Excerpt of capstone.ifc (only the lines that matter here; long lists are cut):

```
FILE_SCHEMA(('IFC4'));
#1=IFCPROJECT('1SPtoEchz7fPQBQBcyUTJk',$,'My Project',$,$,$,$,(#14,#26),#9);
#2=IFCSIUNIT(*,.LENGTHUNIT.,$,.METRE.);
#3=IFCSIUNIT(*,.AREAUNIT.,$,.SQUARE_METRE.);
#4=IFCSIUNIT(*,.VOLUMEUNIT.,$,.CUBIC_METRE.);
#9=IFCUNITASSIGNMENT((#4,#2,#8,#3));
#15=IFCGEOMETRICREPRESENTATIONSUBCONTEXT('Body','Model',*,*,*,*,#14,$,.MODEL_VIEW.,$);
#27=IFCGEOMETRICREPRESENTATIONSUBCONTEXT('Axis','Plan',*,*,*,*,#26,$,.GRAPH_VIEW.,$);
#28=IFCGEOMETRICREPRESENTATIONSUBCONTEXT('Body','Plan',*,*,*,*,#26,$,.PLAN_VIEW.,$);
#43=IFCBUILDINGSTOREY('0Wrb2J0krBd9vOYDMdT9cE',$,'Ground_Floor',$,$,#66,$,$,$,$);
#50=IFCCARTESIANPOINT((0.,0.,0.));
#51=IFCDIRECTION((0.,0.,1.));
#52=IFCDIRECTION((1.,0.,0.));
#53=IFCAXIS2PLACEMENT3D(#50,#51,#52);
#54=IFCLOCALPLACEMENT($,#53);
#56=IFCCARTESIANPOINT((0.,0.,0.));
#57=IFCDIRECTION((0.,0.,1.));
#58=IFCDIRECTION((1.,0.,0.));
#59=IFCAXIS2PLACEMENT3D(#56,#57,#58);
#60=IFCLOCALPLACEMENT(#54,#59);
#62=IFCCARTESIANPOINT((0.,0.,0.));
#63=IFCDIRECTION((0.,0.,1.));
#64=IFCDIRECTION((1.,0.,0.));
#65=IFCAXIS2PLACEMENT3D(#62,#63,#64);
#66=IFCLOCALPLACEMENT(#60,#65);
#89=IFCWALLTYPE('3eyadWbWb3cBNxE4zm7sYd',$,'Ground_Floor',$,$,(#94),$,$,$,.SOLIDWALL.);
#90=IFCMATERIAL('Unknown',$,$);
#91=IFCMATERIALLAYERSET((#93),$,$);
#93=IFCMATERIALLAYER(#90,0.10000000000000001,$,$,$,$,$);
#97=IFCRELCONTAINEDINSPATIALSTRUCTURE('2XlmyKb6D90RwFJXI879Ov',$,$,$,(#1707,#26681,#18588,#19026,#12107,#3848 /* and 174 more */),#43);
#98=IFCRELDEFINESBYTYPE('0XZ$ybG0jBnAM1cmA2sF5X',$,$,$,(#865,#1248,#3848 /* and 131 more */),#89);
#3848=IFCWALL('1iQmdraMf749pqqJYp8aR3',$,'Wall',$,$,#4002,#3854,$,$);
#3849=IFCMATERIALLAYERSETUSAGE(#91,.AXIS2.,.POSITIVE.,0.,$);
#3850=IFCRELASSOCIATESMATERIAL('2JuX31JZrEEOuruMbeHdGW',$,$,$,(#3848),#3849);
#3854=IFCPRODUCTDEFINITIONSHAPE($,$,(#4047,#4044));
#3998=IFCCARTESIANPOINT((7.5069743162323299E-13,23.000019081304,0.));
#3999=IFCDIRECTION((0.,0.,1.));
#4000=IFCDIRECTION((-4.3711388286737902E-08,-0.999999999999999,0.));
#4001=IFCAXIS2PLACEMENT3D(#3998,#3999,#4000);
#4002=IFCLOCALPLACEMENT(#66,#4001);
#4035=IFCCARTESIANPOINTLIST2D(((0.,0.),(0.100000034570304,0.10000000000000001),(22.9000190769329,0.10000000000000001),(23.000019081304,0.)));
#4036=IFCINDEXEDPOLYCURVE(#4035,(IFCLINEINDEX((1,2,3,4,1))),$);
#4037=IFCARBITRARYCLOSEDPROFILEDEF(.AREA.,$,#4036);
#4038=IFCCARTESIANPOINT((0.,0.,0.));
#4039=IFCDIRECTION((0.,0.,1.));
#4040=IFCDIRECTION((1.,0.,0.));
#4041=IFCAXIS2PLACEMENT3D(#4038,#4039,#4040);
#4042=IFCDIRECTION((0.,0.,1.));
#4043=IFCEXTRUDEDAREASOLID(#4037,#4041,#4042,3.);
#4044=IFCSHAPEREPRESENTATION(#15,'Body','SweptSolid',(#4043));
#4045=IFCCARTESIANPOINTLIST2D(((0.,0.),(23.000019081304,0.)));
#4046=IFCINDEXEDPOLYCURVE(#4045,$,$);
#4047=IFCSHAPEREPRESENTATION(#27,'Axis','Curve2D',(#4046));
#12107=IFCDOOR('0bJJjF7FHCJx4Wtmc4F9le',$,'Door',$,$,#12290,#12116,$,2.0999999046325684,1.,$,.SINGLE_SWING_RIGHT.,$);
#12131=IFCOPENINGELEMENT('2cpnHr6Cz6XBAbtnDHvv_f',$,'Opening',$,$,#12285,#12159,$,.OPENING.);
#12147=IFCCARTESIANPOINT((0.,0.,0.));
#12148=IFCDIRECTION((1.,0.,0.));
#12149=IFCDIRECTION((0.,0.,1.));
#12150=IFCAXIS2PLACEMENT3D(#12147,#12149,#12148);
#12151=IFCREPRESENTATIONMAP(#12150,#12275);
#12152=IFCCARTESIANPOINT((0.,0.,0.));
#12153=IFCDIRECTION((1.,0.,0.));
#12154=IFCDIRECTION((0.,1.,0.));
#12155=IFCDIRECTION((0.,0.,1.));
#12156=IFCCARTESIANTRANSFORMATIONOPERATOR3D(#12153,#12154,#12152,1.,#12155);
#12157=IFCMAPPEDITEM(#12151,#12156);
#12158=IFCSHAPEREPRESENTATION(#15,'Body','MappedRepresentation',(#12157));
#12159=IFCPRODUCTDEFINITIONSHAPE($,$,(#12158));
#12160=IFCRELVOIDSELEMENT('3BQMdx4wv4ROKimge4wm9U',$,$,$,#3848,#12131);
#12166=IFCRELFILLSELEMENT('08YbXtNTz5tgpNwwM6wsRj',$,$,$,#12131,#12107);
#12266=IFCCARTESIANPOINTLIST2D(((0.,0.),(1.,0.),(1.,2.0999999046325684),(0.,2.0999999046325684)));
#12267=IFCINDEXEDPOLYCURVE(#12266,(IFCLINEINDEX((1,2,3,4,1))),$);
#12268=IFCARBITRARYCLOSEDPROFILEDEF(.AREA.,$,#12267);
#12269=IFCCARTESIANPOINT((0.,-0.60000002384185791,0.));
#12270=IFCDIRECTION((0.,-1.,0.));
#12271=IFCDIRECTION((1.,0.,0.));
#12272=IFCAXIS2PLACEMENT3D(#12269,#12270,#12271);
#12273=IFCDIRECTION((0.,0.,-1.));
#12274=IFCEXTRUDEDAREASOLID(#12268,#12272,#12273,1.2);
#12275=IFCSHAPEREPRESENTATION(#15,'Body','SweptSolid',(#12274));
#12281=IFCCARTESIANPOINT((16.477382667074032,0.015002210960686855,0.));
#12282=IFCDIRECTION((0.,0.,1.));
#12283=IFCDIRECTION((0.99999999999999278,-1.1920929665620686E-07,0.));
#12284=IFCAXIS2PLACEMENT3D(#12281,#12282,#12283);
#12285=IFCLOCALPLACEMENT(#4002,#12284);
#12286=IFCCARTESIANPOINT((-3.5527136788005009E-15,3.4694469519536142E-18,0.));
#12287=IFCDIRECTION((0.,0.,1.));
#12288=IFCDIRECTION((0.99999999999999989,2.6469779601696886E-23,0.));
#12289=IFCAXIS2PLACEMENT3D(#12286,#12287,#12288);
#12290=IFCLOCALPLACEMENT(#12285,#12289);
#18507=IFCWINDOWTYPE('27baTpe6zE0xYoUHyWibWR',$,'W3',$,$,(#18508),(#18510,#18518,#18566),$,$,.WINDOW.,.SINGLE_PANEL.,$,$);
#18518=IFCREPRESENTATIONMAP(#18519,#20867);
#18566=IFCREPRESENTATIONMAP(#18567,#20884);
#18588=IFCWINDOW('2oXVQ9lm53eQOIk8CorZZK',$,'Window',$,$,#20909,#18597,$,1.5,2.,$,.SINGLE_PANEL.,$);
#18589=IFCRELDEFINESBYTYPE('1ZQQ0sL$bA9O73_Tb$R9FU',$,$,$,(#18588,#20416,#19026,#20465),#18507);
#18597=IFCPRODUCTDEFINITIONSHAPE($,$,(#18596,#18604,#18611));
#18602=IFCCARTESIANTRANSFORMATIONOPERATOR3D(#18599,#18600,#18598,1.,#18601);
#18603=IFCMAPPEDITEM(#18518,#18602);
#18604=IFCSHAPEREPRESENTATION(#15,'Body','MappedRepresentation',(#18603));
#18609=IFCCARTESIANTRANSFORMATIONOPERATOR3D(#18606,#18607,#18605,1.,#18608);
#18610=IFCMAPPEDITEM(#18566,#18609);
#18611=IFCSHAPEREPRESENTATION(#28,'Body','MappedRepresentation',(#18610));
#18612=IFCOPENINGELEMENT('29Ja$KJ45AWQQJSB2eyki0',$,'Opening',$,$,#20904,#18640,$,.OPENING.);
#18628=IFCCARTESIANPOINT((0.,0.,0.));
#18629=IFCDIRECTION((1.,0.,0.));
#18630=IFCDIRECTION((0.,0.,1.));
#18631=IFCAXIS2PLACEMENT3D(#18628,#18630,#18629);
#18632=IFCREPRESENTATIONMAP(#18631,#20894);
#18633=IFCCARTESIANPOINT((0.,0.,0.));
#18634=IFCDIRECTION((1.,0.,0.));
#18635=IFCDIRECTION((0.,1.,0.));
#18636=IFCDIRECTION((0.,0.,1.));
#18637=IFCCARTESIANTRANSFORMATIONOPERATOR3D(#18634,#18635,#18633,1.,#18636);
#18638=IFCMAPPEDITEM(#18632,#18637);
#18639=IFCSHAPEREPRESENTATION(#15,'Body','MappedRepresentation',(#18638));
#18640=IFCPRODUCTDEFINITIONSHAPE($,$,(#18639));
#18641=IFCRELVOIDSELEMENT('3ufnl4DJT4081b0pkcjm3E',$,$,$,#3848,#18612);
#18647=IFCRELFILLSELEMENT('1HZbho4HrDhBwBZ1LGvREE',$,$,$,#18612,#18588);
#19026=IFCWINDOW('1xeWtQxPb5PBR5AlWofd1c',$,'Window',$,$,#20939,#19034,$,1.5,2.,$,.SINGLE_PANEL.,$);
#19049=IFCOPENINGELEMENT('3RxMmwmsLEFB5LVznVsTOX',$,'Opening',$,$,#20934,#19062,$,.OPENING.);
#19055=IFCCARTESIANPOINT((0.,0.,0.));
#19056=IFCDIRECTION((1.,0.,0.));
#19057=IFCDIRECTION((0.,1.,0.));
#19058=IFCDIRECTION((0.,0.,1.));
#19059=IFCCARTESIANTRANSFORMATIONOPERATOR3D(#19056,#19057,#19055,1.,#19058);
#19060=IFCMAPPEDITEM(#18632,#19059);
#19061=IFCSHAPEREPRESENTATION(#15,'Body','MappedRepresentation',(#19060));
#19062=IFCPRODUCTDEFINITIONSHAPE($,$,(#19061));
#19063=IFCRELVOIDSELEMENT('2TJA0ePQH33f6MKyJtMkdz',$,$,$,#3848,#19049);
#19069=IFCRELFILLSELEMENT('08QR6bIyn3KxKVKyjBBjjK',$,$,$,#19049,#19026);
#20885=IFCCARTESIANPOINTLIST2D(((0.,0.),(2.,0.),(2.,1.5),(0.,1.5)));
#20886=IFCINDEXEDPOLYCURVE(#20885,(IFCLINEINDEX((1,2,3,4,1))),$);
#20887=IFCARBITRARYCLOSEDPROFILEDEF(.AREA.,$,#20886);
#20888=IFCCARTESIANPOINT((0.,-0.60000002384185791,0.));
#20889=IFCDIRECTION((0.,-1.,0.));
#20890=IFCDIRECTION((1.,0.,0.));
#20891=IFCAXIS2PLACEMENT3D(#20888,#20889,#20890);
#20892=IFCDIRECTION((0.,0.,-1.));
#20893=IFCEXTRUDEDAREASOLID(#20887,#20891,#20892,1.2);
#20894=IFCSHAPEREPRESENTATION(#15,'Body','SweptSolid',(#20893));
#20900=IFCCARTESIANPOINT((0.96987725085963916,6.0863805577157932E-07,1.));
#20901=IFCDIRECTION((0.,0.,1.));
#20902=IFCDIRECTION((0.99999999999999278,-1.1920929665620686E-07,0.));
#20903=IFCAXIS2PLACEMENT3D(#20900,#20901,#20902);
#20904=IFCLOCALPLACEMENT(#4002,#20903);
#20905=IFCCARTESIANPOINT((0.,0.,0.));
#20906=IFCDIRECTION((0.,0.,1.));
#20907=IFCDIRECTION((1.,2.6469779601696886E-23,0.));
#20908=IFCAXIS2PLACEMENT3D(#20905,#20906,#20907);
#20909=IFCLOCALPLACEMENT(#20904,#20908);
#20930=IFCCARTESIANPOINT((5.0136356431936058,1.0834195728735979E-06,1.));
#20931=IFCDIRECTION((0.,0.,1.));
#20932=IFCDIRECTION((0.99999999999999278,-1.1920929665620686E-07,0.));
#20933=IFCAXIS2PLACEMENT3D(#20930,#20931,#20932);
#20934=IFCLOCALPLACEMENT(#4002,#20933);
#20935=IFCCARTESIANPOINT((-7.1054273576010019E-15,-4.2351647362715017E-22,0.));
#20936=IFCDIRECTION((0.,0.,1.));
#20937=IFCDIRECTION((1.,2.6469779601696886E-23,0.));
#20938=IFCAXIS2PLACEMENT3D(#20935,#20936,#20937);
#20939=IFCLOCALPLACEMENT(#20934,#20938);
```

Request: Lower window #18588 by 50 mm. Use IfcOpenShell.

```python
import numpy as np
import ifcopenshell
import ifcopenshell.api.geometry
import ifcopenshell.util.placement
import ifcopenshell.util.unit

model = ifcopenshell.open("capstone.ifc")
unit_scale = ifcopenshell.util.unit.calculate_unit_scale(model)

window = model.by_id(18588)
opening = window.FillsVoids[0].RelatingOpeningElement
dz = -0.05 / unit_scale

shift = np.array([0.0, 0.0, dz])
# The window is placed relative to its opening, so it follows when the opening moves.
matrix = ifcopenshell.util.placement.get_local_placement(opening.ObjectPlacement)
matrix[:3, 3] += shift
ifcopenshell.api.geometry.edit_object_placement(
    model, product=opening, matrix=matrix, is_si=False, should_transform_children=True
)

print(f"moved by {dz * unit_scale:+.3f} m")

model.write("capstone_updated.ifc")
```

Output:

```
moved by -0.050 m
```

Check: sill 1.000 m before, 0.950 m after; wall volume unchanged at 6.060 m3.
